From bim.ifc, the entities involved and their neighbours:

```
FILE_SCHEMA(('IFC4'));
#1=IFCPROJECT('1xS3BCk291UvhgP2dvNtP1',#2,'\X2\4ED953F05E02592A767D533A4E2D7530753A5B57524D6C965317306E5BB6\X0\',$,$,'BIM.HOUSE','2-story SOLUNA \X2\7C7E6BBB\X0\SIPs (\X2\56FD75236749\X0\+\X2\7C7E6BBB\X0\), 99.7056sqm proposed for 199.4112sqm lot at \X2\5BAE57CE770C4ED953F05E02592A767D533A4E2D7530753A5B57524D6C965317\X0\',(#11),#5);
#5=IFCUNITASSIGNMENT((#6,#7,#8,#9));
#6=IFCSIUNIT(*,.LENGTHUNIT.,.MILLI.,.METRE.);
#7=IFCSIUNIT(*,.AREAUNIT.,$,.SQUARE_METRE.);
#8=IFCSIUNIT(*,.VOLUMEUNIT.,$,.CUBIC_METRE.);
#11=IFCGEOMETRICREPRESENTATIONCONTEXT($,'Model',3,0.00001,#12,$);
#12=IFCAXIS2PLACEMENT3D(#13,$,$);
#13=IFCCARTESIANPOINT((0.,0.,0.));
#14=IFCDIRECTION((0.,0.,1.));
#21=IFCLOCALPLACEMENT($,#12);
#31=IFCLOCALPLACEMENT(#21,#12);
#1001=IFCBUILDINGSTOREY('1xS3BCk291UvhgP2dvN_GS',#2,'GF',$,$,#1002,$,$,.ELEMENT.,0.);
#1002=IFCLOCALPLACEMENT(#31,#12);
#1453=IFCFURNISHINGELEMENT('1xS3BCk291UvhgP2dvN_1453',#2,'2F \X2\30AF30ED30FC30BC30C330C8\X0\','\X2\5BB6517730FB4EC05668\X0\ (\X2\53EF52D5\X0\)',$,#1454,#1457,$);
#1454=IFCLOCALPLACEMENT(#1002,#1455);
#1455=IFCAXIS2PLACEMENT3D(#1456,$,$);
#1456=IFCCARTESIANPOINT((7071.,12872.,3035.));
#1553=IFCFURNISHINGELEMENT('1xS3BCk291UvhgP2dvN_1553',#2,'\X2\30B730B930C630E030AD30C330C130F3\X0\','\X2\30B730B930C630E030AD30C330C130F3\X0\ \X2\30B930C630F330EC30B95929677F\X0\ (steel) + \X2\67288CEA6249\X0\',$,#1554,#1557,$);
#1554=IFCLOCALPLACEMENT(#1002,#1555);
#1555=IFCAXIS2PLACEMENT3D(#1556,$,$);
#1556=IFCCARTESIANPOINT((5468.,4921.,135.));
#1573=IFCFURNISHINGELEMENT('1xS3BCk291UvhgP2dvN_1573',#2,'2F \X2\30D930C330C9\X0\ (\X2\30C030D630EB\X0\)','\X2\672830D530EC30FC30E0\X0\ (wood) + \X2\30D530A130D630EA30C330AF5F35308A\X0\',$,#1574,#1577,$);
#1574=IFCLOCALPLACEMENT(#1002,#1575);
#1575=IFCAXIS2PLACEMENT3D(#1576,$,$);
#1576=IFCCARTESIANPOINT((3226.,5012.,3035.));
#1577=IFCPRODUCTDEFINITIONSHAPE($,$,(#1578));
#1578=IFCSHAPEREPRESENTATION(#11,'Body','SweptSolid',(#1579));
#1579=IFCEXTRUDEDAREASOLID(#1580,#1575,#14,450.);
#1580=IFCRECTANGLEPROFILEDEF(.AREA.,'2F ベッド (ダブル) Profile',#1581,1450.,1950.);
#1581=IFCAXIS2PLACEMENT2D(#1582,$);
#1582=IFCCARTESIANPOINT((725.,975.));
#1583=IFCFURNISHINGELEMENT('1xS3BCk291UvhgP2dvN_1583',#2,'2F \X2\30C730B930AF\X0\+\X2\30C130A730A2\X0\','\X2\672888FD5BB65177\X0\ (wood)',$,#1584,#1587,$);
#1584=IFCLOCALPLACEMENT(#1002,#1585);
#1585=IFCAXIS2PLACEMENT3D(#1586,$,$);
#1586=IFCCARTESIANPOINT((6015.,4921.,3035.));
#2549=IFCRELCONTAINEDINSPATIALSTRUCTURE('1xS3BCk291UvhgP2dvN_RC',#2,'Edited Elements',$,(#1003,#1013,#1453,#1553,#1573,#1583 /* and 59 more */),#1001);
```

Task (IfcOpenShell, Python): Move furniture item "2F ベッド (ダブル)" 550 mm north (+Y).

```python
import ifcopenshell
import ifcopenshell.api.geometry
import ifcopenshell.util.placement
import ifcopenshell.util.unit

model = ifcopenshell.open("bim.ifc")
unit_scale = ifcopenshell.util.unit.calculate_unit_scale(model)

item = model.by_guid("1xS3BCk291UvhgP2dvN_1573")
matrix = ifcopenshell.util.placement.get_local_placement(item.ObjectPlacement)
matrix[1, 3] += 0.55 / unit_scale
ifcopenshell.api.geometry.edit_object_placement(model, product=item, matrix=matrix, is_si=False)

print(ifcopenshell.util.placement.get_local_placement(item.ObjectPlacement).round(3) + 0.0)

model.write("bim-out.ifc")
```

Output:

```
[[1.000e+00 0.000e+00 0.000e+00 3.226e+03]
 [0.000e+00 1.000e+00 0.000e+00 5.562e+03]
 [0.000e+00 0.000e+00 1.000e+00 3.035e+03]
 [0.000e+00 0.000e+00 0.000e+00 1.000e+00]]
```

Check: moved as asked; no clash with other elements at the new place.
